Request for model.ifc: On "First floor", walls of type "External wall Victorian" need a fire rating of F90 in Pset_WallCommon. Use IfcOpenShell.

First a look at what the model holds.

```python
import ifcopenshell
import ifcopenshell.util.element

model = ifcopenshell.open("model.ifc")
print(model.schema)
storey = next(s for s in model.by_type("IfcBuildingStorey") if s.Name == "First floor")
walls = [e for e in ifcopenshell.util.element.get_decomposition(storey) if e.is_a("IfcWall")]
seen = {}
for e in walls:
    element_type = ifcopenshell.util.element.get_type(e)
    key = (element_type.Name if element_type != e and element_type else None, ifcopenshell.util.element.get_pset(e, "Pset_WallCommon", "FireRating"))
    seen[key] = seen.get(key, 0) + 1
for (name, value), count in sorted(seen.items(), key=str):
    print(count, "x", name, "|", value)
```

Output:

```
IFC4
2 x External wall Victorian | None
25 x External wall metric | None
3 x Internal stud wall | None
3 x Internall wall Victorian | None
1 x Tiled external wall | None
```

```python
import ifcopenshell
import ifcopenshell.api.pset
import ifcopenshell.util.element

model = ifcopenshell.open("model.ifc")

storey = next(s for s in model.by_type("IfcBuildingStorey") if s.Name == "First floor")
walls = [e for e in ifcopenshell.util.element.get_decomposition(storey) if e.is_a("IfcWall")]

count = 0
for e in walls:
    element_type = ifcopenshell.util.element.get_type(e)
    if element_type in (None, e) or element_type.Name != "External wall Victorian":
        continue
    # add_pset returns the element's existing set when there is one.
    pset = ifcopenshell.api.pset.add_pset(model, product=e, name="Pset_WallCommon")
    ifcopenshell.api.pset.edit_pset(model, pset=pset, properties={"FireRating": "F90"})
    count += 1

print(count, "walls updated")

model.write("model_updated.ifc")
```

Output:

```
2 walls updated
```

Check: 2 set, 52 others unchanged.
